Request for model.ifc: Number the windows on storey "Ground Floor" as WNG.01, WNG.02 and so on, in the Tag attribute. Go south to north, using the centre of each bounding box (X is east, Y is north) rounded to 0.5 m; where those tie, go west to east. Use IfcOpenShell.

First a look at what the model holds.

```python
import ifcopenshell
import ifcopenshell.util.element
import ifcopenshell.util.placement

model = ifcopenshell.open("model.ifc")
print(model.schema)
storey = next(s for s in model.by_type("IfcBuildingStorey") if s.Name == "Ground Floor")
windows = [e for e in ifcopenshell.util.element.get_decomposition(storey) if e.is_a("IfcWindow")]
for e in sorted(windows, key=lambda e: e.id()):
    origin = ifcopenshell.util.placement.get_local_placement(e.ObjectPlacement)[:3, 3]
    print(e.id(), e.Tag, e.Name, origin.round(2) + 0.0, sep=" | ")
```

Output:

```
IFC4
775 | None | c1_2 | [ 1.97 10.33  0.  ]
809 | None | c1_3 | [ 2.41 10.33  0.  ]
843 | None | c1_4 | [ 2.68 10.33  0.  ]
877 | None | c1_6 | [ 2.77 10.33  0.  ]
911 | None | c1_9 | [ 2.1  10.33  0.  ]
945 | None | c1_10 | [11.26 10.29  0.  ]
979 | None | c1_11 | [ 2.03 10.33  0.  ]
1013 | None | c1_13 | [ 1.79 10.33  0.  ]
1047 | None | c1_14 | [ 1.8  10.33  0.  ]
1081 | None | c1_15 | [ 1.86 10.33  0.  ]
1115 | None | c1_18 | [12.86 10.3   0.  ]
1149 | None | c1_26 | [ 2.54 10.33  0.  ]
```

```python
import ifcopenshell
import ifcopenshell.geom
import ifcopenshell.util.element
import ifcopenshell.util.shape

model = ifcopenshell.open("model.ifc")
settings = ifcopenshell.geom.settings()
settings.set("use-world-coords", True)


def centre(element):
    shape = ifcopenshell.geom.create_shape(settings, element)
    return ifcopenshell.util.shape.get_bbox_centroid(shape.geometry)


storey = next(s for s in model.by_type("IfcBuildingStorey") if s.Name == "Ground Floor")
windows = [e for e in ifcopenshell.util.element.get_decomposition(storey) if e.is_a("IfcWindow")]

# Insertion points can sit at a corner or the storey origin, so sort by the geometry (in metres).
centres = {e: centre(e) for e in windows}
windows.sort(key=lambda e: (round(centres[e][1] / 0.5), centres[e][0]))

for i, e in enumerate(windows, start=1):
    number = f"WNG.{i:02d}"
    e.Tag = number
    print(e.id(), number)

model.write("model_updated.ifc")
```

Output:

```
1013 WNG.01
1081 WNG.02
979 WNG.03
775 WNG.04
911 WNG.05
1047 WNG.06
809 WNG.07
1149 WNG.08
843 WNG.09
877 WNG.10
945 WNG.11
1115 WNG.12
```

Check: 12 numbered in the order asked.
